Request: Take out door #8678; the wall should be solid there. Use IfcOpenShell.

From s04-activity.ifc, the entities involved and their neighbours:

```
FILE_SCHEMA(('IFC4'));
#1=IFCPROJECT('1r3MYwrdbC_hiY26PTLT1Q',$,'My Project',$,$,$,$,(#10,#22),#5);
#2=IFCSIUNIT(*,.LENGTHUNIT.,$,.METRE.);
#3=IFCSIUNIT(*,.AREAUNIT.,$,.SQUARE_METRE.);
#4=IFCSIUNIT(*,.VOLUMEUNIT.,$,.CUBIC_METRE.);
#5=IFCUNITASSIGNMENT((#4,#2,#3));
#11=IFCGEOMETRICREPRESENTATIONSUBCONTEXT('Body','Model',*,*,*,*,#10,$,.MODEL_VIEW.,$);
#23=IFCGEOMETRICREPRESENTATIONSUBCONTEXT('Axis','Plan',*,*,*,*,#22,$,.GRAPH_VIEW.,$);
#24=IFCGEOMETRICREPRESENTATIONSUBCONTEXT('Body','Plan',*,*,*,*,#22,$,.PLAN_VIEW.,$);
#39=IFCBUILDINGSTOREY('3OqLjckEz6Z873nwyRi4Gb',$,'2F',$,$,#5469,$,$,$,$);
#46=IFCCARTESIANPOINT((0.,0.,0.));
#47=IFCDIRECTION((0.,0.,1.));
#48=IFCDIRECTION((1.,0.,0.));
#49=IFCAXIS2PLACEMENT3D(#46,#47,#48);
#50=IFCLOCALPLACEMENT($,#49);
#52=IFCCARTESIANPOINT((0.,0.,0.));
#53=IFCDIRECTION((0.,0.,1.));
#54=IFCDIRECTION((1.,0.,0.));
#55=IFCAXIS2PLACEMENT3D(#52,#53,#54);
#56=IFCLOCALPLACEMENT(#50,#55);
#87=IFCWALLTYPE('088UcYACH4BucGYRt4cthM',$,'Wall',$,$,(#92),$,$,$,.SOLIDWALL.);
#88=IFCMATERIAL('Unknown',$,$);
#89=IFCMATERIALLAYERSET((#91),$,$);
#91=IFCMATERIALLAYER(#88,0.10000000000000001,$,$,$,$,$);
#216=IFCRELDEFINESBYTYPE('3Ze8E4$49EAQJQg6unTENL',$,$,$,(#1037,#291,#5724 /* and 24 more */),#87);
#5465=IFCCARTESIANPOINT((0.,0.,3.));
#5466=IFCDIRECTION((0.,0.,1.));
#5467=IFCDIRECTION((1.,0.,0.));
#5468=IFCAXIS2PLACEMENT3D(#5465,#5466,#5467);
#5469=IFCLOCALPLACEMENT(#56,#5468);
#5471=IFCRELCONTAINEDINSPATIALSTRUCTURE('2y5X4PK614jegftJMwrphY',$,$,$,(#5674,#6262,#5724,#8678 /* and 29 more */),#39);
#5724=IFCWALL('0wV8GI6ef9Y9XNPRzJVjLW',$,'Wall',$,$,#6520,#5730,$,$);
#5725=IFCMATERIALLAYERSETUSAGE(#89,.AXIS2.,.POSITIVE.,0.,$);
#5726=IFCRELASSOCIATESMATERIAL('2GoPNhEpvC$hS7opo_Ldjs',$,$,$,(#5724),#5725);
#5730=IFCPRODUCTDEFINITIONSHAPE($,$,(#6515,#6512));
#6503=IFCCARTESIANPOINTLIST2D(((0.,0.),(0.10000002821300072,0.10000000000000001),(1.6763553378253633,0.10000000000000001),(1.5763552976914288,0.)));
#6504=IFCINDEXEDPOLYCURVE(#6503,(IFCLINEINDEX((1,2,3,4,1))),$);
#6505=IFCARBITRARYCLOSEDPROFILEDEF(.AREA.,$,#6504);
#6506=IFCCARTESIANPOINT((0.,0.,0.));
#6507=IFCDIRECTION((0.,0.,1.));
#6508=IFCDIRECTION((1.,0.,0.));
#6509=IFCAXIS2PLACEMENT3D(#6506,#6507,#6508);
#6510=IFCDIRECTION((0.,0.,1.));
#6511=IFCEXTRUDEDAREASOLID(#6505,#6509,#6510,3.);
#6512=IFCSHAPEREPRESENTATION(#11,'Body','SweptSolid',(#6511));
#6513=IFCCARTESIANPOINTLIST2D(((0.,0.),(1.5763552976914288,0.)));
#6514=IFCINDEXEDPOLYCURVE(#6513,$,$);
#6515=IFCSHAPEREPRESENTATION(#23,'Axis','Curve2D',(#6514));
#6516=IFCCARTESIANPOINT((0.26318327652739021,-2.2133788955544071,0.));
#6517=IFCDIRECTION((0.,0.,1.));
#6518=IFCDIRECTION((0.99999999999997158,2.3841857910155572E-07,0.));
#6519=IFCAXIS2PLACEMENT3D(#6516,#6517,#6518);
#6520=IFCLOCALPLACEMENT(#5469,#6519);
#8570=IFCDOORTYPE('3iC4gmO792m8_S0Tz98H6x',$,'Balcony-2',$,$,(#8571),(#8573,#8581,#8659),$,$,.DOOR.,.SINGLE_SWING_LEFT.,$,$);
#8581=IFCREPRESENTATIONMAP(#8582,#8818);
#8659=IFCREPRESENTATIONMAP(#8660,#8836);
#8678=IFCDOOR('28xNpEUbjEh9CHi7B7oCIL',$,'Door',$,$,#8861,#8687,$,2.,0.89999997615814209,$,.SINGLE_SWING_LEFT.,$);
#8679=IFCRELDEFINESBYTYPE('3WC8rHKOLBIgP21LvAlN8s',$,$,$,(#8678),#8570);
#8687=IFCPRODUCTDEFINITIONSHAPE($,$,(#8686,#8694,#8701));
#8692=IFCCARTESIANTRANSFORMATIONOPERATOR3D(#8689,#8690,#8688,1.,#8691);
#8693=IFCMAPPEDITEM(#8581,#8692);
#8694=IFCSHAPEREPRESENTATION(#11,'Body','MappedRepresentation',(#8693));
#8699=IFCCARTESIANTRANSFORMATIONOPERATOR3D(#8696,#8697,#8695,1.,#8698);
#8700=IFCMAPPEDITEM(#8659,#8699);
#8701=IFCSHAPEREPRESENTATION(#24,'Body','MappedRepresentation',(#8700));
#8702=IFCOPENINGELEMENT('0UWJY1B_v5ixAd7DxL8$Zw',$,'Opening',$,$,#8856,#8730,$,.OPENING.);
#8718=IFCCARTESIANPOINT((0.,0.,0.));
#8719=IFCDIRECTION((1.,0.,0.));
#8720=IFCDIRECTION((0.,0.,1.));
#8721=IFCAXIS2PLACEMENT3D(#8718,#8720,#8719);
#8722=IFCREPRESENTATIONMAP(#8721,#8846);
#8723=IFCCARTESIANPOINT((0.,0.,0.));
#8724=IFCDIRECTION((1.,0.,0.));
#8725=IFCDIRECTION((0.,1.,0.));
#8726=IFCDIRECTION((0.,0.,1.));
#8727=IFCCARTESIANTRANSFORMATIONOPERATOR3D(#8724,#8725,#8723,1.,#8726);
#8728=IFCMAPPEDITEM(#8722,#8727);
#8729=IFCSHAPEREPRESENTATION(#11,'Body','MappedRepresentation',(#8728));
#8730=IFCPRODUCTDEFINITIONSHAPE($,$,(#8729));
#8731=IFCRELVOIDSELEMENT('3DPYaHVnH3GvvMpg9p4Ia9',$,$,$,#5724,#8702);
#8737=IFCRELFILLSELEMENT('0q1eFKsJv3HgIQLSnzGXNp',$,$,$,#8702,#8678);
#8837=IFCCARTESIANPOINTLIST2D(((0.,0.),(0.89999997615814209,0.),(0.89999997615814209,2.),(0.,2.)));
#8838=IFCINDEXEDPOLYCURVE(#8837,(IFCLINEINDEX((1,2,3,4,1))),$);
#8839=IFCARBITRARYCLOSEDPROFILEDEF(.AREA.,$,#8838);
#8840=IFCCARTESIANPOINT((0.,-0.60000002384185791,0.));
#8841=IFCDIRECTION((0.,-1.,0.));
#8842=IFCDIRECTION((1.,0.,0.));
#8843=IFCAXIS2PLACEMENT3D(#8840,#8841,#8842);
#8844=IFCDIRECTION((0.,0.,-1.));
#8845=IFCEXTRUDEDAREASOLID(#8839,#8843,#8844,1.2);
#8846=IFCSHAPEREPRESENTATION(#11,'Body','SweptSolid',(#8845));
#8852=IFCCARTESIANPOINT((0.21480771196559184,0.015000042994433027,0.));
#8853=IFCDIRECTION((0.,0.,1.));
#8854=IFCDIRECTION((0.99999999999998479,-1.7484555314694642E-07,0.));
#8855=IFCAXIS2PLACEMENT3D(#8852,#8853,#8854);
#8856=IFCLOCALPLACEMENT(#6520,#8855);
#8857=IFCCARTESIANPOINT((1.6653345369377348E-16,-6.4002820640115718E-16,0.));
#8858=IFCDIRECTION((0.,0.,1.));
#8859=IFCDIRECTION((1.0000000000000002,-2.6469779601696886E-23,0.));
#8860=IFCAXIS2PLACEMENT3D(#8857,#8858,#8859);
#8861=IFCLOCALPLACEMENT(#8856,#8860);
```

```python
import ifcopenshell
import ifcopenshell.api.feature
import ifcopenshell.api.root
import ifcopenshell.geom
import ifcopenshell.util.shape

model = ifcopenshell.open("s04-activity.ifc")
settings = ifcopenshell.geom.settings()


def volume(element):
    """Net volume in cubic metres, openings subtracted."""
    shape = ifcopenshell.geom.create_shape(settings, element)
    return ifcopenshell.util.shape.get_volume(shape.geometry)


door = model.by_guid("28xNpEUbjEh9CHi7B7oCIL")
opening = door.FillsVoids[0].RelatingOpeningElement
wall = opening.VoidsElements[0].RelatingBuildingElement
before = volume(wall)

ifcopenshell.api.root.remove_product(model, product=door)
ifcopenshell.api.feature.remove_feature(model, feature=opening)

after = volume(wall)

print(f"wall volume {before:.3f} -> {after:.3f} m3")

model.write("s04-activity_updated.ifc")
```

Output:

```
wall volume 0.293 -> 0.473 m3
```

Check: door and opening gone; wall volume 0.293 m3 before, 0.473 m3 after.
